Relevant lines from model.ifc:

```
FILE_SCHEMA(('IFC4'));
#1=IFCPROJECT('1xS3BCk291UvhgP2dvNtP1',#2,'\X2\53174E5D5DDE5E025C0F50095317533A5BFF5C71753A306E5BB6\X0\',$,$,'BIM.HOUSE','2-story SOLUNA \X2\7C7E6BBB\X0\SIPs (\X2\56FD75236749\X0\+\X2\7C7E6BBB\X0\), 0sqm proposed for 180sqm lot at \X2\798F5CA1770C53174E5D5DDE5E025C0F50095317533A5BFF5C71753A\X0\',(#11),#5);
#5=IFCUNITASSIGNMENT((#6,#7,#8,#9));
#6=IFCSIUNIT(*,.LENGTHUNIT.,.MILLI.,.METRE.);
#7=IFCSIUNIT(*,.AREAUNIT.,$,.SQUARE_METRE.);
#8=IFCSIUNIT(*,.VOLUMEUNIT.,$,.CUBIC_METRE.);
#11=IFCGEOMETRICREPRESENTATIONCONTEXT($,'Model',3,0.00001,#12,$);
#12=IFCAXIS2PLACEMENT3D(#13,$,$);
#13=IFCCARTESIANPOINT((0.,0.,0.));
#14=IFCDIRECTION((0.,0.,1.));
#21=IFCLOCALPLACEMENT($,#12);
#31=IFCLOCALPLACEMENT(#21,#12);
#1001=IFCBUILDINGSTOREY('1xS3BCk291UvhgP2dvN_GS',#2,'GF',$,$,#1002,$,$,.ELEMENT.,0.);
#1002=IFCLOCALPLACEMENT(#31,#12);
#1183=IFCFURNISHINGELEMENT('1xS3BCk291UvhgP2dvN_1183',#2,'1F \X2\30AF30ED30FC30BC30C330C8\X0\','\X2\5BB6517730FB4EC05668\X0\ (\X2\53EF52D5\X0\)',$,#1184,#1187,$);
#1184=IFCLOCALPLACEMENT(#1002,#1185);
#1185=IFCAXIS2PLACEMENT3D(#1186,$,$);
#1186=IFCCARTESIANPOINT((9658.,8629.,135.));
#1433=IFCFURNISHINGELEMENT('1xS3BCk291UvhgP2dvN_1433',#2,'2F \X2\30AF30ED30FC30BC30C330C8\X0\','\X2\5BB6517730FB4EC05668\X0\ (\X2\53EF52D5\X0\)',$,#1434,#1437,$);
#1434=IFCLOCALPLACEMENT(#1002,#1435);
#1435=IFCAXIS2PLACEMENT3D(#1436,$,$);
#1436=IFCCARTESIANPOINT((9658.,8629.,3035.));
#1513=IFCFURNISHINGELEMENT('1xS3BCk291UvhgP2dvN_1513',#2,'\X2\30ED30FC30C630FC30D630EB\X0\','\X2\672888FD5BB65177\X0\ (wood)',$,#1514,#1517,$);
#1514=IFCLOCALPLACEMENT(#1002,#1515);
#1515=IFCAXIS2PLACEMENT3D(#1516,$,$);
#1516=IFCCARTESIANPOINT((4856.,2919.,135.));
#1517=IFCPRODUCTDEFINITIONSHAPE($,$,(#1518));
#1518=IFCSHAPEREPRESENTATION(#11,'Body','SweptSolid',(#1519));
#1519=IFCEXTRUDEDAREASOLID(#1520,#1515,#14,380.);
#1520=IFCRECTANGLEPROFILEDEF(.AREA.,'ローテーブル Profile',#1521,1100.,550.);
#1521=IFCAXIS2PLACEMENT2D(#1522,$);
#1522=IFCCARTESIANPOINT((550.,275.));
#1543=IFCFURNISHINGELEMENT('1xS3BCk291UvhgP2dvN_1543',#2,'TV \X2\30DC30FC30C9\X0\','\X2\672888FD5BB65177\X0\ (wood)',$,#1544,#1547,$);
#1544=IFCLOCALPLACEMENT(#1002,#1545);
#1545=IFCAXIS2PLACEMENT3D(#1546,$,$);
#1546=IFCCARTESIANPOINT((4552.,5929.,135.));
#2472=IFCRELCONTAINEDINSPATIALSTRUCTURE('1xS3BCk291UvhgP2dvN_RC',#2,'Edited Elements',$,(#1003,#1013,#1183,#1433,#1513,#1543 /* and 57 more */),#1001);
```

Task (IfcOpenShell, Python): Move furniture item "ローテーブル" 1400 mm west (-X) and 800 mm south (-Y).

```python
import ifcopenshell
import ifcopenshell.api.geometry
import ifcopenshell.util.placement
import ifcopenshell.util.unit

model = ifcopenshell.open("model.ifc")
unit_scale = ifcopenshell.util.unit.calculate_unit_scale(model)

item = model.by_guid("1xS3BCk291UvhgP2dvN_1513")
matrix = ifcopenshell.util.placement.get_local_placement(item.ObjectPlacement)
matrix[0, 3] -= 1.4 / unit_scale
matrix[1, 3] -= 0.8 / unit_scale
ifcopenshell.api.geometry.edit_object_placement(model, product=item, matrix=matrix, is_si=False)

print(ifcopenshell.util.placement.get_local_placement(item.ObjectPlacement).round(3) + 0.0)

model.write("model_edited.ifc")
```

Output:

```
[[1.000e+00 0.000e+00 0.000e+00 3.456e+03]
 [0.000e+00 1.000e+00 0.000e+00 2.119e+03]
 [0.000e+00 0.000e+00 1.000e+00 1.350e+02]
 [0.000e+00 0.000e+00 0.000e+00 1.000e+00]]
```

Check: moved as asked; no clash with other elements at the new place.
